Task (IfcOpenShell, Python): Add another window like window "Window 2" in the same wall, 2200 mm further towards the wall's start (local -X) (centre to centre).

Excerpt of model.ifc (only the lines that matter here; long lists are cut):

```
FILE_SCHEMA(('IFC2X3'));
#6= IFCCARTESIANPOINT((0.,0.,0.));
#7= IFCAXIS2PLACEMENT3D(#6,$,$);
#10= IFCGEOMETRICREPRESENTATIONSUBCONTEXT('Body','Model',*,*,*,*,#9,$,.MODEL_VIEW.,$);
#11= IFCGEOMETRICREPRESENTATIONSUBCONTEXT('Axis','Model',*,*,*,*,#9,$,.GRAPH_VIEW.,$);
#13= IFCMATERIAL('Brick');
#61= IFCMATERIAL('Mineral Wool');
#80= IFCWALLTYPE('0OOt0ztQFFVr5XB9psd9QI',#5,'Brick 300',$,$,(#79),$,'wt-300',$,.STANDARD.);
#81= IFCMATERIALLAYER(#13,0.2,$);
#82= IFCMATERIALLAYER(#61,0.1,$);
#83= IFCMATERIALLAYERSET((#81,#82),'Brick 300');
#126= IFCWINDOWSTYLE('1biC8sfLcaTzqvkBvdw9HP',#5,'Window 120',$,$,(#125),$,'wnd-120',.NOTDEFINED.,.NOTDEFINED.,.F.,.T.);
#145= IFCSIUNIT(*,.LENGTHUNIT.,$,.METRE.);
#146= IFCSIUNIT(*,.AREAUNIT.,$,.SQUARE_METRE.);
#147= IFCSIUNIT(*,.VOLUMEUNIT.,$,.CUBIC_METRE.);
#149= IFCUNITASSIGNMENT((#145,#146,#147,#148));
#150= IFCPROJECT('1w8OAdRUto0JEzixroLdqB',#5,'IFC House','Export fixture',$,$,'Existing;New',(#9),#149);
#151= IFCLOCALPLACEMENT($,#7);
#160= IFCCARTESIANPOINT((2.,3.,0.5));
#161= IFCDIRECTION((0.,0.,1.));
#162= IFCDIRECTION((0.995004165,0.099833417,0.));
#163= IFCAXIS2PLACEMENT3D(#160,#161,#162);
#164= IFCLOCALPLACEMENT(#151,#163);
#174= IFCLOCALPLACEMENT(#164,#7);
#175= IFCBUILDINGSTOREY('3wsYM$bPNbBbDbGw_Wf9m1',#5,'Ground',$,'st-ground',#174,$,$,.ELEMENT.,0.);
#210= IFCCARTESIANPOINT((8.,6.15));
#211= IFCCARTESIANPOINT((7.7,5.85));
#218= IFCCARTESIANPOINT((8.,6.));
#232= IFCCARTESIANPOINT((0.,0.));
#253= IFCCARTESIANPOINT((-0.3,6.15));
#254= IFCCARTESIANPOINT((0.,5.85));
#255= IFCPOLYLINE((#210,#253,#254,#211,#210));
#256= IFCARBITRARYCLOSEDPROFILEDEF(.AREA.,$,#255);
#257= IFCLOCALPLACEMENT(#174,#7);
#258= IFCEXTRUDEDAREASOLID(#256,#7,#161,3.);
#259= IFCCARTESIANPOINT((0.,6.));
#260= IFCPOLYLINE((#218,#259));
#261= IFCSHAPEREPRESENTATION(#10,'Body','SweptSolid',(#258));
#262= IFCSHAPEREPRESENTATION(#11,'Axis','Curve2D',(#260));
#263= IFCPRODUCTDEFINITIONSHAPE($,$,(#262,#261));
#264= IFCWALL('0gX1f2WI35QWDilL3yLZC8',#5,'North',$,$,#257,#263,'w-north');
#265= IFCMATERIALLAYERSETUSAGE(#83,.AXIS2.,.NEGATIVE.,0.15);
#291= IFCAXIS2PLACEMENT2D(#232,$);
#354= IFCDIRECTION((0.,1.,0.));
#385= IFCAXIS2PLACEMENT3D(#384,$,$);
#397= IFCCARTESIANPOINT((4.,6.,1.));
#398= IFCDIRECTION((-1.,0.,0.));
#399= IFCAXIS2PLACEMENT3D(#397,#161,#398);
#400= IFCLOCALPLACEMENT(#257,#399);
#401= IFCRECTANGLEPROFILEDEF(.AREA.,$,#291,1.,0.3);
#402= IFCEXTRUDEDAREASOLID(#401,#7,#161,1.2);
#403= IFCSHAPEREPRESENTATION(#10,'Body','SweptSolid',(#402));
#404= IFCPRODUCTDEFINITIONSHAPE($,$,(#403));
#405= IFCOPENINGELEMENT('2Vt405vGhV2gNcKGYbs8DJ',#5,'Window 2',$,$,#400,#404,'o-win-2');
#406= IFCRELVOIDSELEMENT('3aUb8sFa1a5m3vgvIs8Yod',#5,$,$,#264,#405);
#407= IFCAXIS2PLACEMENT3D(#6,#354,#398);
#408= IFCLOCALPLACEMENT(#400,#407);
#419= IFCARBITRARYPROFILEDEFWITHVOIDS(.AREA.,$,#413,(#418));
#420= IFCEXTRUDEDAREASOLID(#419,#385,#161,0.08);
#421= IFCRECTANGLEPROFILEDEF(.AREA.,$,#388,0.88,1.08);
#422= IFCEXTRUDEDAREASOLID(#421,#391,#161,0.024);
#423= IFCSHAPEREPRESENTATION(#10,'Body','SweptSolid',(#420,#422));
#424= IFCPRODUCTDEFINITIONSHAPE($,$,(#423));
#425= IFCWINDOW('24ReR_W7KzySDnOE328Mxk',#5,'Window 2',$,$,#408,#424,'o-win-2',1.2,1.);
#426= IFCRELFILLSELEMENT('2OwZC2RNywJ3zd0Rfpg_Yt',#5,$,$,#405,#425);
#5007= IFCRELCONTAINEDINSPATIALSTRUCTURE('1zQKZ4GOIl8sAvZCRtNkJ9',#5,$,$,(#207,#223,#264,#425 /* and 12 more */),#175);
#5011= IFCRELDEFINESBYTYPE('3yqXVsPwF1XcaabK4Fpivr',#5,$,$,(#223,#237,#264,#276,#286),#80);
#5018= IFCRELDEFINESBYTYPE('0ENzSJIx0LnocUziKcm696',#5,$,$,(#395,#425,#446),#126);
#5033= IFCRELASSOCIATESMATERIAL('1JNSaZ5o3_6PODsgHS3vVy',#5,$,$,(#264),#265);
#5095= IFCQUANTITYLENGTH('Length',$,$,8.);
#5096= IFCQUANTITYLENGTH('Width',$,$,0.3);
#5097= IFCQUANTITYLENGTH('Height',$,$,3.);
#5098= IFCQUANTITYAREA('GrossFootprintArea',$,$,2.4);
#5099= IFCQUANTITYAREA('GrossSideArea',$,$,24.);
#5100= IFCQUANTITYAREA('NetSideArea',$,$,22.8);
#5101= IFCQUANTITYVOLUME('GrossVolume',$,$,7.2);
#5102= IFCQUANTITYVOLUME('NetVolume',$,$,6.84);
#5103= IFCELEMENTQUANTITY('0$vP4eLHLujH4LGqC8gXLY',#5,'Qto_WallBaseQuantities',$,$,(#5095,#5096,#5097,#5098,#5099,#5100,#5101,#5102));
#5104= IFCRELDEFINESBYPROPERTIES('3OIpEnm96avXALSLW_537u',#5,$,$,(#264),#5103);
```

```python
import ifcopenshell
import ifcopenshell.api.feature
import ifcopenshell.api.geometry
import ifcopenshell.api.pset
import ifcopenshell.api.root
import ifcopenshell.geom
import ifcopenshell.util.element
import ifcopenshell.util.placement
import ifcopenshell.util.shape
import ifcopenshell.util.unit

model = ifcopenshell.open("model.ifc")
area_scale = ifcopenshell.util.unit.calculate_unit_scale(model, "AREAUNIT")
volume_scale = ifcopenshell.util.unit.calculate_unit_scale(model, "VOLUMEUNIT")
settings = ifcopenshell.geom.settings()


def volume(element):
    """Net volume in cubic metres, openings subtracted."""
    shape = ifcopenshell.geom.create_shape(settings, element)
    return ifcopenshell.util.shape.get_volume(shape.geometry)


def reuse_history(source, copy):
    """copy_class also copies each property set's owner history, people and application; keep the originals."""
    for rel in copy.IsDefinedBy:
        if rel.is_a("IfcRelDefinesByProperties") and (history := rel.RelatingPropertyDefinition.OwnerHistory):
            rel.RelatingPropertyDefinition.OwnerHistory = source.OwnerHistory
            ifcopenshell.util.element.remove_deep2(model, history)


window = model.by_id(425)
opening = window.FillsVoids[0].RelatingOpeningElement
wall = opening.VoidsElements[0].RelatingBuildingElement
before = volume(wall)
shift = ifcopenshell.util.placement.get_local_placement(wall.ObjectPlacement)[:3, 0] * -2.2

# copy_class copies the void relationship, type, container and properties, but no geometry.
new_opening = ifcopenshell.api.root.copy_class(model, product=opening)
new_opening.Representation = ifcopenshell.util.element.copy_deep(
    model, opening.Representation, exclude=["IfcGeometricRepresentationContext", "IfcRepresentationMap"]
)
new_opening.Tag = None
new_window = ifcopenshell.api.root.copy_class(model, product=window)
new_window.Representation = ifcopenshell.util.element.copy_deep(
    model, window.Representation, exclude=["IfcGeometricRepresentationContext", "IfcRepresentationMap"]
)
new_window.Tag = None
reuse_history(window, new_window)
fills = ifcopenshell.api.feature.add_filling(model, opening=new_opening, element=new_window)
fills.OwnerHistory = new_window.OwnerHistory  # required in IFC2X3

for old, new in ((opening, new_opening), (window, new_window)):
    matrix = ifcopenshell.util.placement.get_local_placement(old.ObjectPlacement)
    matrix[:3, 3] += shift
    ifcopenshell.api.geometry.edit_object_placement(model, product=new, matrix=matrix, is_si=False)

after = volume(wall)
thickness = 0.3  # wall thickness in metres

# Update the wall's stored quantities.
qto = model.by_id(ifcopenshell.util.element.get_pset(wall, "Qto_WallBaseQuantities", should_inherit=False)["id"])
ifcopenshell.api.pset.edit_qto(model, qto=qto, properties={
    "NetSideArea": after / thickness / area_scale,
    "NetVolume": after / volume_scale,
})

print(f"wall volume {before:.3f} -> {after:.3f} m3")

model.write("model_edited.ifc")
```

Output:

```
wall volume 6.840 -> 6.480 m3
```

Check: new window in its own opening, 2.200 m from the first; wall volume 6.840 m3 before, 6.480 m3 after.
